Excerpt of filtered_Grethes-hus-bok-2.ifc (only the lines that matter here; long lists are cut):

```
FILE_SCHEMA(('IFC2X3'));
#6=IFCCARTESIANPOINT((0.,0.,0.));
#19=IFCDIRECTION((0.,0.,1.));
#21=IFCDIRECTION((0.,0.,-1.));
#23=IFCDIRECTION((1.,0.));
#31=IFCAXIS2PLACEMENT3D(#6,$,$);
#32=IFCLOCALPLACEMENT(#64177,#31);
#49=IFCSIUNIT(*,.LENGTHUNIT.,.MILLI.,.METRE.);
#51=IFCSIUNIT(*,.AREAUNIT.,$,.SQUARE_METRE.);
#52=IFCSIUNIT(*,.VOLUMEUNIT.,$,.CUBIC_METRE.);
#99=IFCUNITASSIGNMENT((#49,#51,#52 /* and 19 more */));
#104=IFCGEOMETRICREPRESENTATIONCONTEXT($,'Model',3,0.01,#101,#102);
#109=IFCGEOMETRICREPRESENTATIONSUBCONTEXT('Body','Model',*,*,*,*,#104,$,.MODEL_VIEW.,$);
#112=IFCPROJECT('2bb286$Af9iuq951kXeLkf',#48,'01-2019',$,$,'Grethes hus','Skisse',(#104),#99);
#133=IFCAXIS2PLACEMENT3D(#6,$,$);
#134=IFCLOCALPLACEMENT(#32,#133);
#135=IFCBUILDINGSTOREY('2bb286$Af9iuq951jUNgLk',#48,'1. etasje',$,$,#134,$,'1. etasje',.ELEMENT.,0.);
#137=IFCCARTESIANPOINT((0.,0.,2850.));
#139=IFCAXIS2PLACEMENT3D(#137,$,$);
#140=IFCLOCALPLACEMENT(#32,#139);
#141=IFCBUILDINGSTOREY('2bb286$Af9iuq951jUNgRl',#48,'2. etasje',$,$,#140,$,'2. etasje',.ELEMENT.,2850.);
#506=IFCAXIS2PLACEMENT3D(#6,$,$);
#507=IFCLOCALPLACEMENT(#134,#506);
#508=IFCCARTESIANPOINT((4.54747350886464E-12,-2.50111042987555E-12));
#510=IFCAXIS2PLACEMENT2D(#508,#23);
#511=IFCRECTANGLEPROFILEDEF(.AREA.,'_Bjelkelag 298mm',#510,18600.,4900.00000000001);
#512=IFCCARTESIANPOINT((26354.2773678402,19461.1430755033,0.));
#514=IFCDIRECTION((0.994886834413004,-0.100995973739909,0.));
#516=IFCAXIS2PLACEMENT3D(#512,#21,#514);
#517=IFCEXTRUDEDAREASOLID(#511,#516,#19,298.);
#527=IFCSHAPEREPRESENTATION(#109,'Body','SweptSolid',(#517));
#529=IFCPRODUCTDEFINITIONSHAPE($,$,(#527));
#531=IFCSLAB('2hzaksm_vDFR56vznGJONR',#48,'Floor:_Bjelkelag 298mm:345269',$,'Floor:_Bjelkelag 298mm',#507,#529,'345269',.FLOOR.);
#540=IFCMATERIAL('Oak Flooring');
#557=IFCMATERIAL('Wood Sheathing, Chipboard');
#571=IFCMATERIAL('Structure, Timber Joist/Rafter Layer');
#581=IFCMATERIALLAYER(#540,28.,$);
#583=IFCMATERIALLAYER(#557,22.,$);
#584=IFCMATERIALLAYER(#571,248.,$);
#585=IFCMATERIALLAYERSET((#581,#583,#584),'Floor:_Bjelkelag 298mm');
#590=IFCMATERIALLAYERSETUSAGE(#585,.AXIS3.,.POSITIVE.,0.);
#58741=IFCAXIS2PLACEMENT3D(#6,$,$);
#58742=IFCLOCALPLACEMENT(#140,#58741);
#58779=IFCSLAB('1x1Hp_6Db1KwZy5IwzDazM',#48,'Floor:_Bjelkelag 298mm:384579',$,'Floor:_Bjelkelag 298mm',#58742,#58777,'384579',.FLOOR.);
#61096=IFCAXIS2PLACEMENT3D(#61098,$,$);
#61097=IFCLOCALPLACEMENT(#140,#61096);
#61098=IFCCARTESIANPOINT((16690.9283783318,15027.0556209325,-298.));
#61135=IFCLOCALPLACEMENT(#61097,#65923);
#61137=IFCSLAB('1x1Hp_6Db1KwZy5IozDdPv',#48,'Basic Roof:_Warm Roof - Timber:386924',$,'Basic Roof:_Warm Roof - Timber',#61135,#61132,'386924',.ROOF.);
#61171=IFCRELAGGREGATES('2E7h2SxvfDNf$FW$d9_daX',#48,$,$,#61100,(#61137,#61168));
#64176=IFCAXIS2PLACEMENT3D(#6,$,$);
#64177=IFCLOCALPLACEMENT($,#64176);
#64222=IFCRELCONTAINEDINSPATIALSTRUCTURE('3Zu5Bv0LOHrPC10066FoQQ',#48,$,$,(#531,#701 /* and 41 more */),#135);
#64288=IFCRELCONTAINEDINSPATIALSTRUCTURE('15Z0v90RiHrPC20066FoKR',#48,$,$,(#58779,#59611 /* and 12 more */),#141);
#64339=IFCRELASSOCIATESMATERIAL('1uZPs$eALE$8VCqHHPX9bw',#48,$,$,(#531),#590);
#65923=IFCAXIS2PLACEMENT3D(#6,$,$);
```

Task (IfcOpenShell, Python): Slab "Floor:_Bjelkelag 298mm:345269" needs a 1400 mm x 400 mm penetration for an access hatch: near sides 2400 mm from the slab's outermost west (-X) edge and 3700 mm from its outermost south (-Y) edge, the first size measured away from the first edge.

```python
import numpy as np
import ifcopenshell
import ifcopenshell.api.feature
import ifcopenshell.api.geometry
import ifcopenshell.api.root
import ifcopenshell.geom
import ifcopenshell.util.placement
import ifcopenshell.util.representation
import ifcopenshell.util.shape
import ifcopenshell.util.unit

model = ifcopenshell.open("filtered_Grethes-hus-bok-2.ifc")
unit_scale = ifcopenshell.util.unit.calculate_unit_scale(model)
settings = ifcopenshell.geom.settings()


def volume(element):
    """Net volume in cubic metres, openings subtracted."""
    shape = ifcopenshell.geom.create_shape(settings, element)
    return ifcopenshell.util.shape.get_volume(shape.geometry)


slab = model.by_guid("2hzaksm_vDFR56vznGJONR")
before = volume(slab)

# Extent in the slab's own axes, in metres. The edges named are its -X and -Y sides.
slab_shape = ifcopenshell.geom.create_shape(settings, slab)
vertices = ifcopenshell.util.shape.get_vertices(slab_shape.geometry)
x_min, y_min, bottom = vertices.min(axis=0)
top = vertices[:, 2].max()

opening = ifcopenshell.api.root.create_entity(model, ifc_class="IfcOpeningElement", name="Access hatch opening")
context = ifcopenshell.util.representation.get_context(model, "Model", "Body", "MODEL_VIEW")
width, depth = 1.4, 0.4
outline = [(0.0, 0.0), (width, 0.0), (width, depth), (0.0, depth), (0.0, 0.0)]
# Overshoot both faces by 50 mm so the cut is clean.
shape = ifcopenshell.api.geometry.add_slab_representation(
    model, context=context, depth=top - bottom + 0.1, polyline=outline
)
ifcopenshell.api.geometry.assign_representation(model, product=opening, representation=shape)

matrix = ifcopenshell.util.placement.get_local_placement(slab.ObjectPlacement)
matrix[:, 3] = matrix @ np.append(np.array([x_min + 2.4, y_min + 3.7, bottom - 0.05]) / unit_scale, 1.0)
ifcopenshell.api.geometry.edit_object_placement(model, product=opening, matrix=matrix, is_si=False)
ifcopenshell.api.feature.add_feature(model, feature=opening, element=slab)

after = volume(slab)

print(f"slab volume {before:.3f} -> {after:.3f} m3")

model.write("filtered_Grethes-hus-bok-2-out.ifc")
```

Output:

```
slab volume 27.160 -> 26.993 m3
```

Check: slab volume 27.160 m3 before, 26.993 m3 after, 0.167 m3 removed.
